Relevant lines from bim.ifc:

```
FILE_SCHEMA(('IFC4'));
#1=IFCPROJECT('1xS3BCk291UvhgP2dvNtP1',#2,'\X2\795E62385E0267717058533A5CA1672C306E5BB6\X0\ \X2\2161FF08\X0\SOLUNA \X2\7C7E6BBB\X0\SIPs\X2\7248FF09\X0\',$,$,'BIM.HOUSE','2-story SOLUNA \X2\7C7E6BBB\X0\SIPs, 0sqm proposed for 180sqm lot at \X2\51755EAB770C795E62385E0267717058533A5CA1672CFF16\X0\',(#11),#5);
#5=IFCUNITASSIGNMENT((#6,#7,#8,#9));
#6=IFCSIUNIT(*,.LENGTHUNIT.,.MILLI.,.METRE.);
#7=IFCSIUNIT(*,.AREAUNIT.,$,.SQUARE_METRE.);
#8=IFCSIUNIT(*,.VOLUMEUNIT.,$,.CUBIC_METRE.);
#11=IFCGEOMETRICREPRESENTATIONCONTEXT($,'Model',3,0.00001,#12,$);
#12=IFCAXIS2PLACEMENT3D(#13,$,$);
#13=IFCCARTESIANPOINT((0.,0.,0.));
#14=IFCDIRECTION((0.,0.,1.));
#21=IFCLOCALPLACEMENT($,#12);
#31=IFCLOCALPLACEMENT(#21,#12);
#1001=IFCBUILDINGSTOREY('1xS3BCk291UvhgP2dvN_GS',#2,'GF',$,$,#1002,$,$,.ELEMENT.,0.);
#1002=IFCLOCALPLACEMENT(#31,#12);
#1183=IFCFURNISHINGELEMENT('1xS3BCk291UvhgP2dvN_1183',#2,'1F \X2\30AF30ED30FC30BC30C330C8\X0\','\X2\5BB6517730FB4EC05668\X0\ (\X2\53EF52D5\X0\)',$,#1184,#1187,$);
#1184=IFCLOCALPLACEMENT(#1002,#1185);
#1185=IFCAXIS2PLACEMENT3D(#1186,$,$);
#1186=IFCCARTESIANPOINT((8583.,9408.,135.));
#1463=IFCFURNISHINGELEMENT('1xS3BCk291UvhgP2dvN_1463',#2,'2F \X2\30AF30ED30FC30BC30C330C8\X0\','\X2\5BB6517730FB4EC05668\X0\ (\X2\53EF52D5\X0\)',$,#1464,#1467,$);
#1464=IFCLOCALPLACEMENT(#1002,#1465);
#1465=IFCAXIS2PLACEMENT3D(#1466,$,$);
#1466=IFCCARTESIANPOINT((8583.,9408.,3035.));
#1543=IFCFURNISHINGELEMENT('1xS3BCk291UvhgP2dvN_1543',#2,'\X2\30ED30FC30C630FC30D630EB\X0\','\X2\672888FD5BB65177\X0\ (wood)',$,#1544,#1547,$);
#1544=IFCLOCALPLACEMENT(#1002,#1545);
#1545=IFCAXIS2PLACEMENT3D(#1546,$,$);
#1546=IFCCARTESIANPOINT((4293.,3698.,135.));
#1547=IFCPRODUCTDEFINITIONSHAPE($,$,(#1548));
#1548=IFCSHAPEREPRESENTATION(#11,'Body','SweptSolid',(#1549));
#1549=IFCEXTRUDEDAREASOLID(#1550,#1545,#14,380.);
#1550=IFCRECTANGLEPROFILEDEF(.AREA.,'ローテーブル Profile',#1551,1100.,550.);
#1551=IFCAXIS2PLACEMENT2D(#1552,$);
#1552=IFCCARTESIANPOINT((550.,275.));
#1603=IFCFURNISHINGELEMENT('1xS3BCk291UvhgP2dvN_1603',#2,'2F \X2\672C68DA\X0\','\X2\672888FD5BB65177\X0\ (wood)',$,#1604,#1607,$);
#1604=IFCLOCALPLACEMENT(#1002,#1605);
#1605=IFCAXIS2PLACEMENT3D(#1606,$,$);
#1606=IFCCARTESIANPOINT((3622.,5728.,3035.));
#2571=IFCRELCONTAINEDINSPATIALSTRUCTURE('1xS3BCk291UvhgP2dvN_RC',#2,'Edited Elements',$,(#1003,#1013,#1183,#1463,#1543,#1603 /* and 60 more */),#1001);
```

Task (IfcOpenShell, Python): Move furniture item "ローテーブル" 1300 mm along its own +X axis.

```python
import ifcopenshell
import ifcopenshell.api.geometry
import ifcopenshell.util.placement
import ifcopenshell.util.unit

model = ifcopenshell.open("bim.ifc")
unit_scale = ifcopenshell.util.unit.calculate_unit_scale(model)

item = model.by_guid("1xS3BCk291UvhgP2dvN_1543")
matrix = ifcopenshell.util.placement.get_local_placement(item.ObjectPlacement)
matrix[:3, 3] += matrix[:3, 0] * 1.3 / unit_scale
ifcopenshell.api.geometry.edit_object_placement(model, product=item, matrix=matrix, is_si=False)

print(ifcopenshell.util.placement.get_local_placement(item.ObjectPlacement).round(3) + 0.0)

model.write("bim_edited.ifc")
```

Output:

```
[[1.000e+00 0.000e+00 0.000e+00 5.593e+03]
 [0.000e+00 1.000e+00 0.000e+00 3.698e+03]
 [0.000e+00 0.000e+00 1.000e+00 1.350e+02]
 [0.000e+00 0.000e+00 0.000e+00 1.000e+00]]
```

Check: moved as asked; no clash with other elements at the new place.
